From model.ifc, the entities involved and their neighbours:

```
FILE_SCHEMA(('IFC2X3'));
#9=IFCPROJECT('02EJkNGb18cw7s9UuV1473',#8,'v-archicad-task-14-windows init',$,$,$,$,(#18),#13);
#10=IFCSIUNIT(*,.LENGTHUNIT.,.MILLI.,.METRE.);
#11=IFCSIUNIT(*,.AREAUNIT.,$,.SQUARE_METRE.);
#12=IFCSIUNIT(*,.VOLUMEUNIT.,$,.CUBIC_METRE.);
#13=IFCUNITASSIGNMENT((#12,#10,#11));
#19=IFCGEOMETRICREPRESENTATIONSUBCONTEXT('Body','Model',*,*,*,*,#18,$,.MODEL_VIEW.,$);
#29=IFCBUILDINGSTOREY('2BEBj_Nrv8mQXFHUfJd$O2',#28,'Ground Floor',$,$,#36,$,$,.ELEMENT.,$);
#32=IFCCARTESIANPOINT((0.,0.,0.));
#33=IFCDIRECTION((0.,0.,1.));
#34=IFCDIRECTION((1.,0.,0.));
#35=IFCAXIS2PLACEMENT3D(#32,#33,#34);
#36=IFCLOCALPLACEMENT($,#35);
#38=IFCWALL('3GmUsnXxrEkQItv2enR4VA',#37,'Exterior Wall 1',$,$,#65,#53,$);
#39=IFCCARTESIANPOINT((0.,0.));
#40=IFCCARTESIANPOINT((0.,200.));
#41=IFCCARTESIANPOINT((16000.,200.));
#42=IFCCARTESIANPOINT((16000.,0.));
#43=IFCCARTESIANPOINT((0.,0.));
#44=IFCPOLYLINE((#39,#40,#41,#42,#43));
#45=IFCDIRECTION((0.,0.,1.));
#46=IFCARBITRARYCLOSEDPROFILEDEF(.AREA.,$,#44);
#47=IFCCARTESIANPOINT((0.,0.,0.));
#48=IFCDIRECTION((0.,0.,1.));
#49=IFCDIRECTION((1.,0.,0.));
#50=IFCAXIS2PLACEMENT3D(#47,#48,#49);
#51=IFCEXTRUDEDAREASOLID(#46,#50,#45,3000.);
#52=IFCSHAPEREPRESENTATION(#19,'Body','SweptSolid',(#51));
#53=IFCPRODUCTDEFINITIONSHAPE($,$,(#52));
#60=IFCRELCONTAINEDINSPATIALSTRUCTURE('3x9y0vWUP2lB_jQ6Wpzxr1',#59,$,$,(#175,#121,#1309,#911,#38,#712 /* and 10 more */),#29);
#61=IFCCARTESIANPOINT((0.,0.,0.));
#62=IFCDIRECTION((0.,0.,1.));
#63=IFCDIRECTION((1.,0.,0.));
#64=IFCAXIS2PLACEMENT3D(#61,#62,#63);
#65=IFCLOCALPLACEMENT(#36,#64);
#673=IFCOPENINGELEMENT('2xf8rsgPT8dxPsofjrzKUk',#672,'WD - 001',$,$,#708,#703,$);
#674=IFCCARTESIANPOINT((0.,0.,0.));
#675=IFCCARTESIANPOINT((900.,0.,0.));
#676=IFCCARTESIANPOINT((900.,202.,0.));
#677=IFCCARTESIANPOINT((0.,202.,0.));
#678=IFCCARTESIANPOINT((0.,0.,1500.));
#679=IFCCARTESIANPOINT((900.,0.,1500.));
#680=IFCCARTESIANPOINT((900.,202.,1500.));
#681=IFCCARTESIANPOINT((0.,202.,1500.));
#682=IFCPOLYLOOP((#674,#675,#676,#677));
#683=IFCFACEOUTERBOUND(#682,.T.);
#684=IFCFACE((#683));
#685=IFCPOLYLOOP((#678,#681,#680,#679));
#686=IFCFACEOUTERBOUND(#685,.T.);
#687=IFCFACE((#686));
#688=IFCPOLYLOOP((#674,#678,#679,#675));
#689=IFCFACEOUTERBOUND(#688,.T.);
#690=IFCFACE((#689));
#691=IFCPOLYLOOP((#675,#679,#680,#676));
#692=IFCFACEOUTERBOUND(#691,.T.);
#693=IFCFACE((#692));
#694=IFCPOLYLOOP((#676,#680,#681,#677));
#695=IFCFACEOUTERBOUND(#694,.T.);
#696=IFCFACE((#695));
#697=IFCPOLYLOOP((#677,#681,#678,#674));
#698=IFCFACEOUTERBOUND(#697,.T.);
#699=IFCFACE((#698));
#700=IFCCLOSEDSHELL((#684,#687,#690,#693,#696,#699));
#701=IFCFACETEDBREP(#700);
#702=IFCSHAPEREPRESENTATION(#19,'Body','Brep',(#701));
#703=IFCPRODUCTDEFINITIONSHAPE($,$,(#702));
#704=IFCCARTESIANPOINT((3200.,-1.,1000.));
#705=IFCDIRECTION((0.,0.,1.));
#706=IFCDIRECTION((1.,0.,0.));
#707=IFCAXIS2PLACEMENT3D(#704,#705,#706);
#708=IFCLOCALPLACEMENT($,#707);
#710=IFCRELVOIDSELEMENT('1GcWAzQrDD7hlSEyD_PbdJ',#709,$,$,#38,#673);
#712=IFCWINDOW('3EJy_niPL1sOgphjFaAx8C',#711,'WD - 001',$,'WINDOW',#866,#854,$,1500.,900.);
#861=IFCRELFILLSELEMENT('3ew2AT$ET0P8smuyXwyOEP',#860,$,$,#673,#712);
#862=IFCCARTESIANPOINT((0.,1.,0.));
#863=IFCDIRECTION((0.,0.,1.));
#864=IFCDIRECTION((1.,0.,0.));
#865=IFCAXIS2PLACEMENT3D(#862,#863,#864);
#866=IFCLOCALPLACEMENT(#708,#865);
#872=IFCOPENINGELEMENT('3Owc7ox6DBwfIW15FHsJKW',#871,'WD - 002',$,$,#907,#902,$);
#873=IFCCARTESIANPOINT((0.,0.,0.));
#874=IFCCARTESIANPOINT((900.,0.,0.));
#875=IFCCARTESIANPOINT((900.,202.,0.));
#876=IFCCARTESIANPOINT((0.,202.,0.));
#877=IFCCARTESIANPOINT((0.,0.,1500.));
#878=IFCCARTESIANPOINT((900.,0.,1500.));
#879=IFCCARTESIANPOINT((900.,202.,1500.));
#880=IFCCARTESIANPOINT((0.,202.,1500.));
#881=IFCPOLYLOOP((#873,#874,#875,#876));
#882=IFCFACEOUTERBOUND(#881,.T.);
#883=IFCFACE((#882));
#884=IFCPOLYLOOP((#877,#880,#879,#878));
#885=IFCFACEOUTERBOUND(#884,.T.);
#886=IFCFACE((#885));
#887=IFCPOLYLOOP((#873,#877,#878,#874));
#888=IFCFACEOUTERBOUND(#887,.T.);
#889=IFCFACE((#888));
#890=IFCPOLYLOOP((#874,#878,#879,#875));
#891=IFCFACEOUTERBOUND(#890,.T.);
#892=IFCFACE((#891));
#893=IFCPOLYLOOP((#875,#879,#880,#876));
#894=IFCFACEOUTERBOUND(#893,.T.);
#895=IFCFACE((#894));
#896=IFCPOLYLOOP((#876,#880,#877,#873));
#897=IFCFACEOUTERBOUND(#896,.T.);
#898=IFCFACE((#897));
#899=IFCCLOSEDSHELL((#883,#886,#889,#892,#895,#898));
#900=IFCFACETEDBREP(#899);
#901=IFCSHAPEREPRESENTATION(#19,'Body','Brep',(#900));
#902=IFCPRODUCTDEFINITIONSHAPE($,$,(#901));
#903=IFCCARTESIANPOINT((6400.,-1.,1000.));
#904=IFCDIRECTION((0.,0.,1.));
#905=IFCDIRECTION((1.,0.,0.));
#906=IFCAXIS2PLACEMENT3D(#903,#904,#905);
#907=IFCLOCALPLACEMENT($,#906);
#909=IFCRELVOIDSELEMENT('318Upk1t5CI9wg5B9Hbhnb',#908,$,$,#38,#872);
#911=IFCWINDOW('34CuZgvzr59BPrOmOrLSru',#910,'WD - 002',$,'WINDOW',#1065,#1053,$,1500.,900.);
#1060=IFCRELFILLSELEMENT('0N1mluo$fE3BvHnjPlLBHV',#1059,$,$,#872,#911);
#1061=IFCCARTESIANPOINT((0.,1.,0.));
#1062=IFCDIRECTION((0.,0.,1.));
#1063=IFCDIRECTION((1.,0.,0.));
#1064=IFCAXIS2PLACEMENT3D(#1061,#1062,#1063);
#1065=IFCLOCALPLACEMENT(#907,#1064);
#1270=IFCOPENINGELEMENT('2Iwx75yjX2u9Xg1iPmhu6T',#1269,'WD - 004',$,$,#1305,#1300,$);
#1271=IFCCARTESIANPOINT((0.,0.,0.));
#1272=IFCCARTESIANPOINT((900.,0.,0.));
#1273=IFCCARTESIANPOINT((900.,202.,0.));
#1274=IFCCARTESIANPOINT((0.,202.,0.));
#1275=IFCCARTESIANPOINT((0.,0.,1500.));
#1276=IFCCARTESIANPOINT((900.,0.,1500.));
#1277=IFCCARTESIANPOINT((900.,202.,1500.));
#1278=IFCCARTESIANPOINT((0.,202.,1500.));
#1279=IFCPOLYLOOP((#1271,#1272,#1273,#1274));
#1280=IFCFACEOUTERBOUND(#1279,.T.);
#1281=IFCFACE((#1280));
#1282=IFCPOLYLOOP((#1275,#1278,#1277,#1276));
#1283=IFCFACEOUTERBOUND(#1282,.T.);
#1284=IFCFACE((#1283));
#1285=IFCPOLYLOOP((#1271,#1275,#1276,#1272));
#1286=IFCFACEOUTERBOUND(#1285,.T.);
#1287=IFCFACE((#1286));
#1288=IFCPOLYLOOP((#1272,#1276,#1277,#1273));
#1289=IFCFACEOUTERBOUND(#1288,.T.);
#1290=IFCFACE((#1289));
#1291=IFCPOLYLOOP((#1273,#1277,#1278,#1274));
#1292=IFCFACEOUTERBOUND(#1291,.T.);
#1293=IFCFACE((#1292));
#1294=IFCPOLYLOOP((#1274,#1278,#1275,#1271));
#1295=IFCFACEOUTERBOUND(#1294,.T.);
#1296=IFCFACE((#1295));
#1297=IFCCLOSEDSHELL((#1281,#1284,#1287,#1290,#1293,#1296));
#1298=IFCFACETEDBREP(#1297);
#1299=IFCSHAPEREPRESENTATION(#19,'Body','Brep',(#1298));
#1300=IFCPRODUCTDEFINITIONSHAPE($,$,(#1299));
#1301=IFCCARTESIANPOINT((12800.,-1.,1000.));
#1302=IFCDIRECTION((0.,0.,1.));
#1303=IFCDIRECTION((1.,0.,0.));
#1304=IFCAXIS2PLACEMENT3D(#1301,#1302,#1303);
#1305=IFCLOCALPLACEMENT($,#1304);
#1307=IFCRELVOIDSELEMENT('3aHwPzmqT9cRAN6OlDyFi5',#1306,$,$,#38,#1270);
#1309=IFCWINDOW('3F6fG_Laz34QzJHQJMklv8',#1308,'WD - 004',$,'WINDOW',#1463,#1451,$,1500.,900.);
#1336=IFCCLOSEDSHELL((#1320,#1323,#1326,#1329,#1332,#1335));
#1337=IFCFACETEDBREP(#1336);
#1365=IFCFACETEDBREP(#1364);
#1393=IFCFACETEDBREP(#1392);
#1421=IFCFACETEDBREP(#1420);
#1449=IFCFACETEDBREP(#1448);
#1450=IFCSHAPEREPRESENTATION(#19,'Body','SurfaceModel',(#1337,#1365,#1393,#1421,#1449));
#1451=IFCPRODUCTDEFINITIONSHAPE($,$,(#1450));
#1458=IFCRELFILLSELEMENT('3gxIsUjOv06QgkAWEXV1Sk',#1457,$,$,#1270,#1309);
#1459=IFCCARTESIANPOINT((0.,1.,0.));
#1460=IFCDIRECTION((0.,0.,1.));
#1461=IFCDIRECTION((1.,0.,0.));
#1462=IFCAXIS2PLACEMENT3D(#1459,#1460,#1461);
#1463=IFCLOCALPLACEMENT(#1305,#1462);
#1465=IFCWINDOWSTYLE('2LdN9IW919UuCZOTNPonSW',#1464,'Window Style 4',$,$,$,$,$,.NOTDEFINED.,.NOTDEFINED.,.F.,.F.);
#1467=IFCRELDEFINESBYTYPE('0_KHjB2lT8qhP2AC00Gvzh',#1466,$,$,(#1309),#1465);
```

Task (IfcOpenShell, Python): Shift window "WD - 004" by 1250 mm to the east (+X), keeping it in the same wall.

```python
import ifcopenshell
import ifcopenshell.api.geometry
import ifcopenshell.util.placement

model = ifcopenshell.open("model.ifc")

window = model.by_id(1309)
opening = window.FillsVoids[0].RelatingOpeningElement
wall = opening.VoidsElements[0].RelatingBuildingElement

wall_matrix = ifcopenshell.util.placement.get_local_placement(wall.ObjectPlacement)
shift = wall_matrix[:3, 0] * 1250.0
before = ifcopenshell.util.placement.get_local_placement(window.ObjectPlacement)[:3, 3].copy()

# The window is placed relative to its opening, so it follows when the opening moves.
matrix = ifcopenshell.util.placement.get_local_placement(opening.ObjectPlacement)
matrix[:3, 3] += shift
ifcopenshell.api.geometry.edit_object_placement(
    model, product=opening, matrix=matrix, is_si=False, should_transform_children=True
)

after = ifcopenshell.util.placement.get_local_placement(window.ObjectPlacement)[:3, 3]
print("window moved by", (after - before).round(3) + 0.0)

model.write("model_rev.ifc")
```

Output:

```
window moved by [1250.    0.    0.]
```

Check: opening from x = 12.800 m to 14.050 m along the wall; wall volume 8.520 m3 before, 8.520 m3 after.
